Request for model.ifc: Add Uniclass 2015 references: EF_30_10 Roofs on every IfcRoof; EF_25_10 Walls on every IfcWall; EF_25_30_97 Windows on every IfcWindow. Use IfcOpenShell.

First a look at what the model holds.

```python
import ifcopenshell

model = ifcopenshell.open("model.ifc")
print(model.schema)
print("classifications:", [c.Name for c in model.by_type("IfcClassification")])
for ifc_class in ("IfcDoor", "IfcRoof", "IfcStair", "IfcWall", "IfcWindow"):
    print(ifc_class, len(model.by_type(ifc_class)))
```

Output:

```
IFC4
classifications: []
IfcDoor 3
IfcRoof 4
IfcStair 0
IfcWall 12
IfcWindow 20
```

```python
import ifcopenshell
import ifcopenshell.api.classification

model = ifcopenshell.open("model.ifc")

system = ifcopenshell.api.classification.add_classification(model, classification="Uniclass 2015")

codes = {
    "IfcRoof": ("EF_30_10", "Roofs"),
    "IfcWall": ("EF_25_10", "Walls"),
    "IfcWindow": ("EF_25_30_97", "Windows"),
}
for ifc_class, (code, name) in codes.items():
    products = model.by_type(ifc_class)
    ifcopenshell.api.classification.add_reference(
        model, products=products, classification=system, identification=code, name=name
    )
    print(code, len(products))

model.write("model_updated.ifc")
```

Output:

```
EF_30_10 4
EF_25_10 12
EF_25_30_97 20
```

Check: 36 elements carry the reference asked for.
